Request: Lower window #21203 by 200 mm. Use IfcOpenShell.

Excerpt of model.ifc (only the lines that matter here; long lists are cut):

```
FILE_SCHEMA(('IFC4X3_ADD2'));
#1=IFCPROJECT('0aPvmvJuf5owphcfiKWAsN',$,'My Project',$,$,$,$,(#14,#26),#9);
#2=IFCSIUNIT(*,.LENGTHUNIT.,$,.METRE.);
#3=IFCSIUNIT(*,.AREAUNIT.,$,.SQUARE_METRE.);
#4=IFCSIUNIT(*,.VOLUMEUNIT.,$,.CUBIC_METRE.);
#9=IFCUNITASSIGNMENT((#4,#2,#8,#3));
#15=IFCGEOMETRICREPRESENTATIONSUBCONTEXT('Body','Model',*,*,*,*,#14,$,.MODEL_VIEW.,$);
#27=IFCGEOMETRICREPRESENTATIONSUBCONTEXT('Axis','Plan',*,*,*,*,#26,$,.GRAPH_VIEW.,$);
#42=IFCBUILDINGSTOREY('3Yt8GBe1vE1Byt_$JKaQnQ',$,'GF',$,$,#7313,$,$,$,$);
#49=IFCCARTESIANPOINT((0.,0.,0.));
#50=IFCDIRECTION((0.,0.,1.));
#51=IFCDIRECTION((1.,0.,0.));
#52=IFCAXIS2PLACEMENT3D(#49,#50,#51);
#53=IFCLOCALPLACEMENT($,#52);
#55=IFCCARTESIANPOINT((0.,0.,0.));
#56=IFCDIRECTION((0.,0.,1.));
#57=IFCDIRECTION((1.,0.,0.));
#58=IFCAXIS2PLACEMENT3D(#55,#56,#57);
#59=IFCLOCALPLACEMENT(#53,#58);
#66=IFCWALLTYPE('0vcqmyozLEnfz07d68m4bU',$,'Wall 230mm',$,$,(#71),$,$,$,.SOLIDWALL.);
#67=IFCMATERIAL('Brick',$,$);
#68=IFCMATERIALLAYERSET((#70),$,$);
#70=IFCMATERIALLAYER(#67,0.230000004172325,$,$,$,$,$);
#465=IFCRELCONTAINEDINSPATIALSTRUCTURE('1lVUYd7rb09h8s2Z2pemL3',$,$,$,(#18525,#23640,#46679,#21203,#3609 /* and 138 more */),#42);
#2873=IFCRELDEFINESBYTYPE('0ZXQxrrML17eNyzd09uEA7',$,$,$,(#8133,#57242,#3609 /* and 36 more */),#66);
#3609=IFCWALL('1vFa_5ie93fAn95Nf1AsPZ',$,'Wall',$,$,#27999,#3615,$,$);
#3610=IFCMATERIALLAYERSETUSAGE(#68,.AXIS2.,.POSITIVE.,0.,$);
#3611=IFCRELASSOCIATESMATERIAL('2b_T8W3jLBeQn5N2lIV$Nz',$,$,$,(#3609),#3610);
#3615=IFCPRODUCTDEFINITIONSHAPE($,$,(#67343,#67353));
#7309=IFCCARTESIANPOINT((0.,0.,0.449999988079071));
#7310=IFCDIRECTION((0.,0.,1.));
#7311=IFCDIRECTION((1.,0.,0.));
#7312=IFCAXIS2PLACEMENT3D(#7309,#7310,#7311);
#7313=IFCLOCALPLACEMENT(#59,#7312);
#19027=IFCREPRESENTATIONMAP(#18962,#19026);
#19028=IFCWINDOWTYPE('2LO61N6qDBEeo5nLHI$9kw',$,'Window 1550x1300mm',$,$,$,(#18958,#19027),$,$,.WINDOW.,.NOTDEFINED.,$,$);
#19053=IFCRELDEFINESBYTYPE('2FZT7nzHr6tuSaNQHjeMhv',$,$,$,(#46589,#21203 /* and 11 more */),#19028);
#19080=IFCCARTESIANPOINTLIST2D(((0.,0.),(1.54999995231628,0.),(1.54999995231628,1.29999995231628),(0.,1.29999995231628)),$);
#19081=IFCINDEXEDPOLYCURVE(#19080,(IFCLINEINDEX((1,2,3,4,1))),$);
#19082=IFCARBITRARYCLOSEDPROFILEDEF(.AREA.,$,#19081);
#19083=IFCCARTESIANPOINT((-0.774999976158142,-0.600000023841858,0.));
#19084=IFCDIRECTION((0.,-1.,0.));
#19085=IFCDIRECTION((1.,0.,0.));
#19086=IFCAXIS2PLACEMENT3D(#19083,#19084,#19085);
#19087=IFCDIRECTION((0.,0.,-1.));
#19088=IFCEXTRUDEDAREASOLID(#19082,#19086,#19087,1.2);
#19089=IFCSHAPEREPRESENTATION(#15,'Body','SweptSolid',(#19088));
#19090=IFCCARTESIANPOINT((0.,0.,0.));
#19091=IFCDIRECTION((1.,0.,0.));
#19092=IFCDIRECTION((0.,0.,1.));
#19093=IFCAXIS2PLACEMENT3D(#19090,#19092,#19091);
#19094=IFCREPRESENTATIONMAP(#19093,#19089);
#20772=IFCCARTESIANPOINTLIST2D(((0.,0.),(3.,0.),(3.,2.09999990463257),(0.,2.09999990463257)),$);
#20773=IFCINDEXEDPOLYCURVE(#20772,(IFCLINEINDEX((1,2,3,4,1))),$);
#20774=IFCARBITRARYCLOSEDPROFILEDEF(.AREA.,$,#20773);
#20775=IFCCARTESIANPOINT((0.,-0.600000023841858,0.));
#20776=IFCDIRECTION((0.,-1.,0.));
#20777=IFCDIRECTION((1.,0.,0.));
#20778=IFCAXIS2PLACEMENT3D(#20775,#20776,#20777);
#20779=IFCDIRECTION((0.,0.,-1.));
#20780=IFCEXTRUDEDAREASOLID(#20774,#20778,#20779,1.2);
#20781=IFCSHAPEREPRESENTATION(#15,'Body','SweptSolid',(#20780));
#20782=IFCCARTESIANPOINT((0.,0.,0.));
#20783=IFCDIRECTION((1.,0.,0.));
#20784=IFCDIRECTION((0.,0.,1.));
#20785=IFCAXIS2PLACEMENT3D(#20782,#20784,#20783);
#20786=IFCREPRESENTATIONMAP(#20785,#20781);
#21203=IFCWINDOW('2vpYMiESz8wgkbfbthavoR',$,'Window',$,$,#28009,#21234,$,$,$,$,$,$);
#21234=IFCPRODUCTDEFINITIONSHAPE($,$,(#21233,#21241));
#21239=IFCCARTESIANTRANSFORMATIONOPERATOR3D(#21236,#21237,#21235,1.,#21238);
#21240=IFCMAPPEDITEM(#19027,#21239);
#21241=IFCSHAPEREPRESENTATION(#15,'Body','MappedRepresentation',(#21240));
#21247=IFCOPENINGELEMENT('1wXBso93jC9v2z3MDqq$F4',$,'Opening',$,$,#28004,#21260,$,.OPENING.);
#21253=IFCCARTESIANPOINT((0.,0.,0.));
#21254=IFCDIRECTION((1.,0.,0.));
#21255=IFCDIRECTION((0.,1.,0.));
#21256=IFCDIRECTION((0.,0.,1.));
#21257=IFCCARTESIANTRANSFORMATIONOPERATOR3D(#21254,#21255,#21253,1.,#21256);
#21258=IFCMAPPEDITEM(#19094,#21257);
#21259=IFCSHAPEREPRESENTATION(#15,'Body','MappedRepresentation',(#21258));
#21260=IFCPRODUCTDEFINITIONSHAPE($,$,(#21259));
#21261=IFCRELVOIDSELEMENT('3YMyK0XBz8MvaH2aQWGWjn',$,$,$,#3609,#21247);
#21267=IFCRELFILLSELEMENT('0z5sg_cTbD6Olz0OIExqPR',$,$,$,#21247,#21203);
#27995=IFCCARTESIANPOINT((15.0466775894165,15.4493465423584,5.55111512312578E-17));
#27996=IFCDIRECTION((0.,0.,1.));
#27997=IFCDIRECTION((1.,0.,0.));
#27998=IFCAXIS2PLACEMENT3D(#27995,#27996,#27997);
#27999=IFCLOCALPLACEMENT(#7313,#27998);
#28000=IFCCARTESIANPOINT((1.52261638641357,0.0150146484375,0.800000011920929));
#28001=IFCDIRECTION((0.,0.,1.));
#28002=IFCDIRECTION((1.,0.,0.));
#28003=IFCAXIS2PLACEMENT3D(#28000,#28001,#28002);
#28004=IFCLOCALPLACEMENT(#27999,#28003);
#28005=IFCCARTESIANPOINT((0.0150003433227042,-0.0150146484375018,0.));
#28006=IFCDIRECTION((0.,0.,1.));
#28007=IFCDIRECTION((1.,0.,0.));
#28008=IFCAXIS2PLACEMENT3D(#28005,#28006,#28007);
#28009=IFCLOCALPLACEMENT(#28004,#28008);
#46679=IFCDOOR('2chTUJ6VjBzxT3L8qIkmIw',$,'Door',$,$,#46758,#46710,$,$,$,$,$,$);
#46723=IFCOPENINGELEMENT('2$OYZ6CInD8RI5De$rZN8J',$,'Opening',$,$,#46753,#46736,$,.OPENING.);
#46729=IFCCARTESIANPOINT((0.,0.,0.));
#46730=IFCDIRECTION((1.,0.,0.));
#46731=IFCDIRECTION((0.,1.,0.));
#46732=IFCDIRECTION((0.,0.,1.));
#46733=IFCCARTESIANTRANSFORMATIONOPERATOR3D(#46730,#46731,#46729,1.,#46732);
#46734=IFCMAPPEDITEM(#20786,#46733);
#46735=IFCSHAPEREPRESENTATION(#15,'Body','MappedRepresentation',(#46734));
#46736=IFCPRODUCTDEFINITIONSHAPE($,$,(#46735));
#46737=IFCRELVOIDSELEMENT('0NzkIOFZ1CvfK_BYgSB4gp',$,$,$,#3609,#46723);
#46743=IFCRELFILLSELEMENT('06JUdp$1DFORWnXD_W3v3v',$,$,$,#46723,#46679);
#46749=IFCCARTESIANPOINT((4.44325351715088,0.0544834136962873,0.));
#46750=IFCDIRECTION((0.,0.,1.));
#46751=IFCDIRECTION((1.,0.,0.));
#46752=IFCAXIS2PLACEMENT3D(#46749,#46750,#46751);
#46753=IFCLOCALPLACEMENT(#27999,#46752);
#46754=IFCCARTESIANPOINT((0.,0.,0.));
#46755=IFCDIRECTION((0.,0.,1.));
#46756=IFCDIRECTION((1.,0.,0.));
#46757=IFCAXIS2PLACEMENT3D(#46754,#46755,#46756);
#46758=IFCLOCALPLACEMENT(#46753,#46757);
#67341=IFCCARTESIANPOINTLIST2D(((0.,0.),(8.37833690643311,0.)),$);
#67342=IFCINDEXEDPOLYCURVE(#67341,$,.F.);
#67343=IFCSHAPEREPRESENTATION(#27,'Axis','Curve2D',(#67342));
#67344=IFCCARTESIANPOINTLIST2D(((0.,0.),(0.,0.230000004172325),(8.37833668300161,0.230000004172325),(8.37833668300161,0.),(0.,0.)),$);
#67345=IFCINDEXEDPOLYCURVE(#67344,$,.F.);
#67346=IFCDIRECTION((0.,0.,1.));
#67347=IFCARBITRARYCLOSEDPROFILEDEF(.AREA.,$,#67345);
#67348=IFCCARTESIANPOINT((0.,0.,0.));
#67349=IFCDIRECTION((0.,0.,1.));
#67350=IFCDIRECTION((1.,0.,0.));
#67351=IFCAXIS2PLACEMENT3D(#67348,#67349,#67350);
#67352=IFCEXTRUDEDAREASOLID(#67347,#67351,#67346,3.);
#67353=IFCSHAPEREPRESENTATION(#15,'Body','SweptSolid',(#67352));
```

```python
import numpy as np
import ifcopenshell
import ifcopenshell.api.geometry
import ifcopenshell.util.placement
import ifcopenshell.util.unit

model = ifcopenshell.open("model.ifc")
unit_scale = ifcopenshell.util.unit.calculate_unit_scale(model)

window = model.by_guid("2vpYMiESz8wgkbfbthavoR")
opening = window.FillsVoids[0].RelatingOpeningElement
dz = -0.2 / unit_scale

shift = np.array([0.0, 0.0, dz])
# The window is placed relative to its opening, so it follows when the opening moves.
matrix = ifcopenshell.util.placement.get_local_placement(opening.ObjectPlacement)
matrix[:3, 3] += shift
ifcopenshell.api.geometry.edit_object_placement(
    model, product=opening, matrix=matrix, is_si=False, should_transform_children=True
)

print(f"moved by {dz * unit_scale:+.3f} m")

model.write("model_rev.ifc")
```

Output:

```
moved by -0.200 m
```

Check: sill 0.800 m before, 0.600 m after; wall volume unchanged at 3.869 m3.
